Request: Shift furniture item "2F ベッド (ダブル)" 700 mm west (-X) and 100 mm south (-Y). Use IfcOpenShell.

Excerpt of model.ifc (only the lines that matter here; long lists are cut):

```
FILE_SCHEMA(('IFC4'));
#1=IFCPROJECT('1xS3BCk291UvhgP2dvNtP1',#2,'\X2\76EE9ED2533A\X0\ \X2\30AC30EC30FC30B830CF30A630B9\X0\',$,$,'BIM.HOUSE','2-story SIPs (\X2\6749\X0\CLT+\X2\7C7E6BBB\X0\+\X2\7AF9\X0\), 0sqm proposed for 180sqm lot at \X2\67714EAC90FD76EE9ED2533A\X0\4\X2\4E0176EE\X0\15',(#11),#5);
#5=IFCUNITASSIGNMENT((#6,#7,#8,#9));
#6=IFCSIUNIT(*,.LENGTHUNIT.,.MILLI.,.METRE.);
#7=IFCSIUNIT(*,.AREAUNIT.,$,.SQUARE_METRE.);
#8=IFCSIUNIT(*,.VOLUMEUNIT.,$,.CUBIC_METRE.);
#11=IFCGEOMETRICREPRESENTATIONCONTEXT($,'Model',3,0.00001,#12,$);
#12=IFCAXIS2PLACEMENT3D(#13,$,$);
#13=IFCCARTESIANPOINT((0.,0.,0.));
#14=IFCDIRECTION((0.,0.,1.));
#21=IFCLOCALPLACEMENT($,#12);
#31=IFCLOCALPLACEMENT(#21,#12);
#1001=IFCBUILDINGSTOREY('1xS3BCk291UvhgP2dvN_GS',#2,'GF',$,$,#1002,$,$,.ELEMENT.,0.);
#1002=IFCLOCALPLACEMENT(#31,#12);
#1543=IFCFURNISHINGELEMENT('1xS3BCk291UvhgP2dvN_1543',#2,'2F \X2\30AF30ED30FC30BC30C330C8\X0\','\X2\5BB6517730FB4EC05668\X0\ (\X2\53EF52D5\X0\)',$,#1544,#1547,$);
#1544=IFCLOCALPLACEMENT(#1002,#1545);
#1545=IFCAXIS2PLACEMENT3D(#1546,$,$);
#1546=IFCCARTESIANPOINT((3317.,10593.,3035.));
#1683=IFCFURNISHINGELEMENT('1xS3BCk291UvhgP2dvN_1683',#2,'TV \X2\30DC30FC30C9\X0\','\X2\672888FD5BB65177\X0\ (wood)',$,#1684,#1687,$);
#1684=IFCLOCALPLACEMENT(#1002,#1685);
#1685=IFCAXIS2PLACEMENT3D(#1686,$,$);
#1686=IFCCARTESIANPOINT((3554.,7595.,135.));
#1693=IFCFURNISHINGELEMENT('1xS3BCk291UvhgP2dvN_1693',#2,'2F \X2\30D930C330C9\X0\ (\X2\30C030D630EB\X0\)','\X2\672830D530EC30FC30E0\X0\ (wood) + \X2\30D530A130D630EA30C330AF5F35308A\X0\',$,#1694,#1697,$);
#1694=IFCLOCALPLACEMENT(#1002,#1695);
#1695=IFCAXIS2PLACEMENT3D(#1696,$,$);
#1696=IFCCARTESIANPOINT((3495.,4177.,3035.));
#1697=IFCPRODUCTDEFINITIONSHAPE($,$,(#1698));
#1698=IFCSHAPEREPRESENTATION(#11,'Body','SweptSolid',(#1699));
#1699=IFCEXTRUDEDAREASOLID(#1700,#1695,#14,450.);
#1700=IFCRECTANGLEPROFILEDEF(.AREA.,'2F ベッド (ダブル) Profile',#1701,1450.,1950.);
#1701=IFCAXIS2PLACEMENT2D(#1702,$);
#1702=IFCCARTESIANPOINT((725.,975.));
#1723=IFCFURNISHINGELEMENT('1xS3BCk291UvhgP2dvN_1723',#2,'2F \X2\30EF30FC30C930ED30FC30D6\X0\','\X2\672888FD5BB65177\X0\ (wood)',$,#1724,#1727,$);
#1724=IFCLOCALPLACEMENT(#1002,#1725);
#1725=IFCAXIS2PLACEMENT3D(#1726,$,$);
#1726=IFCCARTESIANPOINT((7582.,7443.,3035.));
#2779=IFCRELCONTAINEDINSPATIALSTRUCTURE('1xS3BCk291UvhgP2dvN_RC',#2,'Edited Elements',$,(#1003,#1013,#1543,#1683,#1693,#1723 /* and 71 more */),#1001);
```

```python
import ifcopenshell
import ifcopenshell.api.geometry
import ifcopenshell.util.placement
import ifcopenshell.util.unit

model = ifcopenshell.open("model.ifc")
unit_scale = ifcopenshell.util.unit.calculate_unit_scale(model)

item = model.by_guid("1xS3BCk291UvhgP2dvN_1693")
matrix = ifcopenshell.util.placement.get_local_placement(item.ObjectPlacement)
matrix[0, 3] -= 0.7 / unit_scale
matrix[1, 3] -= 0.1 / unit_scale
ifcopenshell.api.geometry.edit_object_placement(model, product=item, matrix=matrix, is_si=False)

print(ifcopenshell.util.placement.get_local_placement(item.ObjectPlacement).round(3) + 0.0)

model.write("model_rev.ifc")
```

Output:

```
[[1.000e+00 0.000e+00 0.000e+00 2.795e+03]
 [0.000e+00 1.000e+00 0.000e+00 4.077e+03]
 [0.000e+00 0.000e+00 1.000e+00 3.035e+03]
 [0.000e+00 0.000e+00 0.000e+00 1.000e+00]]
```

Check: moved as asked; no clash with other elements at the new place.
